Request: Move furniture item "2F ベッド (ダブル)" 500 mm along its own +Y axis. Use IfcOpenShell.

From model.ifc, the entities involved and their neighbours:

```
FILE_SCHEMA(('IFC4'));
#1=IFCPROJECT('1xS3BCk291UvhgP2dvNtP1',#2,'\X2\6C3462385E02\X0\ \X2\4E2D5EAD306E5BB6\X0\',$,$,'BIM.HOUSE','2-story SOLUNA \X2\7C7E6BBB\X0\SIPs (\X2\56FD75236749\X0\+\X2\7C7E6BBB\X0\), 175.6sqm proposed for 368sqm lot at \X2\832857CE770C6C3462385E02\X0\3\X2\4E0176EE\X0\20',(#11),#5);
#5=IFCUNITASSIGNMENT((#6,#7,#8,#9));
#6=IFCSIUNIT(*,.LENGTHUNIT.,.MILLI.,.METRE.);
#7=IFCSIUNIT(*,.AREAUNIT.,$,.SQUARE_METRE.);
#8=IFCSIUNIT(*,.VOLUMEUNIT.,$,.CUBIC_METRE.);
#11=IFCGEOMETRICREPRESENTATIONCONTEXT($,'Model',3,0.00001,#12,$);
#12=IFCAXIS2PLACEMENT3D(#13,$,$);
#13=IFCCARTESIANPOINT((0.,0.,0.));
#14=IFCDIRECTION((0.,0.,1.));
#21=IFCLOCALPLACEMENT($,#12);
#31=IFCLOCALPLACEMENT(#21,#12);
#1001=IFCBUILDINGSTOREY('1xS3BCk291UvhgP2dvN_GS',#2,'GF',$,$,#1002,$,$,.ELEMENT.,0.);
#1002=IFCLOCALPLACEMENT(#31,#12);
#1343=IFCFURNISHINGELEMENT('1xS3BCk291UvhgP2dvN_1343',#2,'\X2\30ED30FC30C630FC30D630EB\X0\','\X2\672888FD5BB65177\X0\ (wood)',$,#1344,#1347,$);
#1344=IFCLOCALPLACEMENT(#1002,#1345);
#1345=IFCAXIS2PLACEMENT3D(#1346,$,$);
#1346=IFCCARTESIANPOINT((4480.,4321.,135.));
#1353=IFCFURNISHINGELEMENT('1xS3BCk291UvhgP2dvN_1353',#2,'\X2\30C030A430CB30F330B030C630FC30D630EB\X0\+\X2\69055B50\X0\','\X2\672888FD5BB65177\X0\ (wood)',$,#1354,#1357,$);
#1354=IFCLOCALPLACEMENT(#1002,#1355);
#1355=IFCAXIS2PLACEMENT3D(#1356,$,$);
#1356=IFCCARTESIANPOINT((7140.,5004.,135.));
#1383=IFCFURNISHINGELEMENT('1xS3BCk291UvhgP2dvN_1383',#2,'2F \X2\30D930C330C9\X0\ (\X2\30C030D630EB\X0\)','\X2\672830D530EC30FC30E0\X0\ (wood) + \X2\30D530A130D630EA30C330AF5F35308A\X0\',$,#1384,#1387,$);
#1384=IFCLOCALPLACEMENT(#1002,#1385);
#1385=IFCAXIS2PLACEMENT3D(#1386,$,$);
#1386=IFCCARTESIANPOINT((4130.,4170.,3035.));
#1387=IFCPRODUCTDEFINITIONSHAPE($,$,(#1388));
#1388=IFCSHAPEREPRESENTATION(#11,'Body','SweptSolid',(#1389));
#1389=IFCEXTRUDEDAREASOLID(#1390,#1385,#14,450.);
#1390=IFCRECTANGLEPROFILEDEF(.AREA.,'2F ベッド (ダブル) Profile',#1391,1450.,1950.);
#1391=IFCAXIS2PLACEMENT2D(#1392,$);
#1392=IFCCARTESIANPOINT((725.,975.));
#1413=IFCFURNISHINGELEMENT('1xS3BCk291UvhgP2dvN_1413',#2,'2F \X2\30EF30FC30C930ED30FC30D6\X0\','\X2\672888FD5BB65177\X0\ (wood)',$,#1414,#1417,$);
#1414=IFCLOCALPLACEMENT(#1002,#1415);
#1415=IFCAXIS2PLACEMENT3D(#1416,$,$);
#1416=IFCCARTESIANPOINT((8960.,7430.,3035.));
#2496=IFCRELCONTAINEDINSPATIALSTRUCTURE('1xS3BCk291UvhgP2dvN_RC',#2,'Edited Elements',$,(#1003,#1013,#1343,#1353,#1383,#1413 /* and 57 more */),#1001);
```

```python
import ifcopenshell
import ifcopenshell.api.geometry
import ifcopenshell.util.placement
import ifcopenshell.util.unit

model = ifcopenshell.open("model.ifc")
unit_scale = ifcopenshell.util.unit.calculate_unit_scale(model)

item = model.by_guid("1xS3BCk291UvhgP2dvN_1383")
matrix = ifcopenshell.util.placement.get_local_placement(item.ObjectPlacement)
matrix[:3, 3] += matrix[:3, 1] * 0.5 / unit_scale
ifcopenshell.api.geometry.edit_object_placement(model, product=item, matrix=matrix, is_si=False)

print(ifcopenshell.util.placement.get_local_placement(item.ObjectPlacement).round(3) + 0.0)

model.write("model_updated.ifc")
```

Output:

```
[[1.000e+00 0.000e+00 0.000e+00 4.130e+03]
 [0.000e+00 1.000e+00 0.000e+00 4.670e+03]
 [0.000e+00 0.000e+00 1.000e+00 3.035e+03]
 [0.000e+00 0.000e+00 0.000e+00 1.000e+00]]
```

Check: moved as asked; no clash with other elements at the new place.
